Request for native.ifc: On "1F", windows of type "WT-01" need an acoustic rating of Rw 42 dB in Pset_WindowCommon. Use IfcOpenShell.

First a look at what the model holds.

```python
import ifcopenshell
import ifcopenshell.util.element

model = ifcopenshell.open("native.ifc")
print(model.schema)
storey = next(s for s in model.by_type("IfcBuildingStorey") if s.Name == "1F")
windows = [e for e in ifcopenshell.util.element.get_decomposition(storey) if e.is_a("IfcWindow")]
seen = {}
for e in windows:
    element_type = ifcopenshell.util.element.get_type(e)
    key = (element_type.Name if element_type != e and element_type else None, ifcopenshell.util.element.get_pset(e, "Pset_WindowCommon", "AcousticRating"))
    seen[key] = seen.get(key, 0) + 1
for (name, value), count in sorted(seen.items(), key=str):
    print(count, "x", name, "|", value)
```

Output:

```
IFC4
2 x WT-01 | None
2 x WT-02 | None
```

```python
import ifcopenshell
import ifcopenshell.api.pset
import ifcopenshell.util.element

model = ifcopenshell.open("native.ifc")

storey = next(s for s in model.by_type("IfcBuildingStorey") if s.Name == "1F")
windows = [e for e in ifcopenshell.util.element.get_decomposition(storey) if e.is_a("IfcWindow")]

count = 0
for e in windows:
    element_type = ifcopenshell.util.element.get_type(e)
    if element_type in (None, e) or element_type.Name != "WT-01":
        continue
    found = ifcopenshell.util.element.get_pset(e, "Pset_WindowCommon", should_inherit=False)
    if found:
        pset = model.by_id(found["id"])
        if len(ifcopenshell.util.element.get_elements_by_pset(pset)) > 1:
            pset = ifcopenshell.api.pset.unshare_pset(model, products=[e], pset=pset)[0]
    else:
        pset = ifcopenshell.api.pset.add_pset(model, product=e, name="Pset_WindowCommon")
    ifcopenshell.api.pset.edit_pset(model, pset=pset, properties={"AcousticRating": "Rw 42 dB"})
    count += 1

print(count, "windows updated")

model.write("native_v2.ifc")
```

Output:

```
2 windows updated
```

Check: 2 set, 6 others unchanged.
